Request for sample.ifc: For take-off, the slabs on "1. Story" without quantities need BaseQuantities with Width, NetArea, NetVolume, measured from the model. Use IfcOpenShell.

First a look at what the model holds.

```python
import ifcopenshell
import ifcopenshell.util.element
import ifcopenshell.util.unit

model = ifcopenshell.open("sample.ifc")
print(model.schema)
for unit_type in ("LENGTHUNIT", "AREAUNIT", "VOLUMEUNIT"):
    print(unit_type, ifcopenshell.util.unit.calculate_unit_scale(model, unit_type))
storey = next(s for s in model.by_type("IfcBuildingStorey") if s.Name == "1. Story")
slabs = [e for e in ifcopenshell.util.element.get_decomposition(storey) if e.is_a("IfcSlab")]
for e in sorted(slabs, key=lambda e: e.id()):
    print(e.id(), e.is_a(), e.Name, list(ifcopenshell.util.element.get_psets(e, qtos_only=True)), sep=" | ")
```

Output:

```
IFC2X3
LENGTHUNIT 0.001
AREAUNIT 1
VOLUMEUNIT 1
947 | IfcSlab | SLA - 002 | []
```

```python
import ifcopenshell
import ifcopenshell.api.pset
import ifcopenshell.geom
import ifcopenshell.util.element
import ifcopenshell.util.shape
import ifcopenshell.util.unit

model = ifcopenshell.open("sample.ifc")
unit_scale = ifcopenshell.util.unit.calculate_unit_scale(model)
area_scale = ifcopenshell.util.unit.calculate_unit_scale(model, "AREAUNIT")
volume_scale = ifcopenshell.util.unit.calculate_unit_scale(model, "VOLUMEUNIT")
settings = ifcopenshell.geom.settings()

storey = next(s for s in model.by_type("IfcBuildingStorey") if s.Name == "1. Story")
slabs = [e for e in ifcopenshell.util.element.get_decomposition(storey) if e.is_a("IfcSlab")]

for e in sorted(slabs, key=lambda e: e.id()):
    if ifcopenshell.util.element.get_psets(e, qtos_only=True, should_inherit=False):
        continue
    # Geometry comes back in metres, in the element's own axes.
    shape = ifcopenshell.geom.create_shape(settings, e)
    values = {
        "Width": ifcopenshell.util.shape.get_z(shape.geometry) / unit_scale,
        "NetArea": ifcopenshell.util.shape.get_footprint_area(shape.geometry) / area_scale,
        "NetVolume": ifcopenshell.util.shape.get_volume(shape.geometry) / volume_scale,
    }
    qto = ifcopenshell.api.pset.add_qto(model, product=e, name="BaseQuantities")
    ifcopenshell.api.pset.edit_qto(model, qto=qto, properties=values)
    print(e.id(), {k: round(v, 3) for k, v in values.items()})

model.write("sample_edited.ifc")
```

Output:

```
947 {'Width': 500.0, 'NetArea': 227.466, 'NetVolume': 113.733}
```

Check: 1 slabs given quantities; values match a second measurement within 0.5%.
